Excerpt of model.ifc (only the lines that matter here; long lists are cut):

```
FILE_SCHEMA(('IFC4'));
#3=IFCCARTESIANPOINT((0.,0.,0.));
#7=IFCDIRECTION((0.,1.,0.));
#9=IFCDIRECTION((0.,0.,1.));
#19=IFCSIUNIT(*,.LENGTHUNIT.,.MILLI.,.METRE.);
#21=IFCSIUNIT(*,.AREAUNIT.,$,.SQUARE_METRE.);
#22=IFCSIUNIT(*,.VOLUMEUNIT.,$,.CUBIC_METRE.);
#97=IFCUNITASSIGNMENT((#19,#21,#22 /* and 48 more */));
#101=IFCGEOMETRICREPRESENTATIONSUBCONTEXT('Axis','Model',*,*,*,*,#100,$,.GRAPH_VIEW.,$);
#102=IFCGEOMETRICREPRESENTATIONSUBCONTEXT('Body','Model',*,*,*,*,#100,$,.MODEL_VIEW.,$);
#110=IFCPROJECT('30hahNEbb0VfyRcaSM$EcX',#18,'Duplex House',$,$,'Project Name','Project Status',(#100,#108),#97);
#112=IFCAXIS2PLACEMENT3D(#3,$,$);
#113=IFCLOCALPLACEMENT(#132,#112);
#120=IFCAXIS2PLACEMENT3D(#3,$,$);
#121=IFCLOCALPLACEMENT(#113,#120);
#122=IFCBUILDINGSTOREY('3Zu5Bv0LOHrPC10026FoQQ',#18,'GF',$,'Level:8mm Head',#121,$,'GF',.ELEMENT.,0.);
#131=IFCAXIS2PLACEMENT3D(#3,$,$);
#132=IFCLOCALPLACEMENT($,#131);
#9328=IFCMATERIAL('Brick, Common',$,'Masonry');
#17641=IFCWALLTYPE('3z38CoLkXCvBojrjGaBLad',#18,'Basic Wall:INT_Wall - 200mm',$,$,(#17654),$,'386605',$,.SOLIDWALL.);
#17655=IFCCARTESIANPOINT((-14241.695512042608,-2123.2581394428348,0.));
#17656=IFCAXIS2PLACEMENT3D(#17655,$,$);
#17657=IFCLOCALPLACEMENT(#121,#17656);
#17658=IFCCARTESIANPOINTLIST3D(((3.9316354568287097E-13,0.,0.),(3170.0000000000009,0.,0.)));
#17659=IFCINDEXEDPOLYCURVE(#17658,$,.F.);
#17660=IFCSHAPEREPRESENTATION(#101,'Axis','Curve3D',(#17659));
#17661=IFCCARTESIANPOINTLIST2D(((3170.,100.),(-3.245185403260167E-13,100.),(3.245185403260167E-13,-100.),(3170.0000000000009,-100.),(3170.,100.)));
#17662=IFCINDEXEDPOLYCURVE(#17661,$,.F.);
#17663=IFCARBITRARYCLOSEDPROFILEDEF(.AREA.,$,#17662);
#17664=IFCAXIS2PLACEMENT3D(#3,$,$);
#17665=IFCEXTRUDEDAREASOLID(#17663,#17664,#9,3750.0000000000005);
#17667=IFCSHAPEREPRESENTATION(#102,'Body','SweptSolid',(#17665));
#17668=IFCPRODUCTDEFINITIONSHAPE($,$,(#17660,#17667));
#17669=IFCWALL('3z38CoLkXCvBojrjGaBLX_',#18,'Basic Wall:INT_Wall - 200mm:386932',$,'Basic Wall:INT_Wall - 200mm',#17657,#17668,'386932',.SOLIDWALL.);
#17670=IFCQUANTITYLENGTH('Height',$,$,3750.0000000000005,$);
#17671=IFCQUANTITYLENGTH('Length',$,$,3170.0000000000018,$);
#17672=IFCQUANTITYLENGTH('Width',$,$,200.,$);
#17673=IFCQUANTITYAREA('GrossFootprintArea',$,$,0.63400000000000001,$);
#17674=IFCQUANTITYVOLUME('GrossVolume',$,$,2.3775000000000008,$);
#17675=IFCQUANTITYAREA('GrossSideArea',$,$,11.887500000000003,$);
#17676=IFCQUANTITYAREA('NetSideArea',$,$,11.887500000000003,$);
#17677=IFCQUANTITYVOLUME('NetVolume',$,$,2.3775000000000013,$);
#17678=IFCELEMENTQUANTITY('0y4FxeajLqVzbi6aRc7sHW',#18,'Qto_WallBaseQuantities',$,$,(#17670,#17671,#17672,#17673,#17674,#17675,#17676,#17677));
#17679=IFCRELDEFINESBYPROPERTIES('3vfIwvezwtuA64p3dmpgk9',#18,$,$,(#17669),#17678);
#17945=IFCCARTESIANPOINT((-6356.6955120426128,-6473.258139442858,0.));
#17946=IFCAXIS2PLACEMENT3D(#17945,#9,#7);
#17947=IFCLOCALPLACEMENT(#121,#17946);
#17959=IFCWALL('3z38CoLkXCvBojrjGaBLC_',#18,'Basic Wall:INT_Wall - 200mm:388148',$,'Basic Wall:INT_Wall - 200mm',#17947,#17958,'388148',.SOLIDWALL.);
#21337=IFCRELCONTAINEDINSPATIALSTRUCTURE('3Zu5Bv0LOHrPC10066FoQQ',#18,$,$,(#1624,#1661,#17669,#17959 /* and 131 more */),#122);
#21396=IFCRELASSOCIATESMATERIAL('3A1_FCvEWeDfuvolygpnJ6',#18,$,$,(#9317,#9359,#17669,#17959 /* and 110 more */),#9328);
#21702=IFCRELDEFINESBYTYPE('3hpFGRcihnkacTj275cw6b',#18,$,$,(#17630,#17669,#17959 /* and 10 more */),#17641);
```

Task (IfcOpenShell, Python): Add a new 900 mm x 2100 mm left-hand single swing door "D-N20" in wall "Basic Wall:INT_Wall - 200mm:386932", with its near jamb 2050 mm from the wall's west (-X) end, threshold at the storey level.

```python
import numpy as np
import ifcopenshell
import ifcopenshell.api.feature
import ifcopenshell.api.geometry
import ifcopenshell.api.pset
import ifcopenshell.api.root
import ifcopenshell.api.spatial
import ifcopenshell.geom
import ifcopenshell.util.element
import ifcopenshell.util.placement
import ifcopenshell.util.representation
import ifcopenshell.util.shape
import ifcopenshell.util.unit

model = ifcopenshell.open("model.ifc")
unit_scale = ifcopenshell.util.unit.calculate_unit_scale(model)
area_scale = ifcopenshell.util.unit.calculate_unit_scale(model, "AREAUNIT")
volume_scale = ifcopenshell.util.unit.calculate_unit_scale(model, "VOLUMEUNIT")
settings = ifcopenshell.geom.settings()


def volume(element):
    """Net volume in cubic metres, openings subtracted."""
    shape = ifcopenshell.geom.create_shape(settings, element)
    return ifcopenshell.util.shape.get_volume(shape.geometry)


wall = model.by_guid("3z38CoLkXCvBojrjGaBLX_")
storey = ifcopenshell.util.element.get_container(wall, ifc_class="IfcBuildingStorey")
context = ifcopenshell.util.representation.get_context(model, "Model", "Body", "MODEL_VIEW")
before = volume(wall)

width, height, from_end, sill = 0.9, 2.1, 2.05, 0.0  # metres

# The wall runs along its own X axis, and the end named is its -X end.
wall_shape = ifcopenshell.geom.create_shape(settings, wall)
x, y, z = ifcopenshell.util.shape.get_vertices(wall_shape.geometry).T
start = x.min() + from_end
face, thickness = float(y.min()), float(y.max() - y.min())
wall_matrix = ifcopenshell.util.placement.get_local_placement(wall.ObjectPlacement)
level = ifcopenshell.util.placement.get_local_placement(storey.ObjectPlacement)[2, 3]


def in_wall(x, y):
    """Placement at x, y metres in the wall's axes, at sill height."""
    matrix = wall_matrix.copy()
    matrix[:, 3] = wall_matrix @ np.array([x / unit_scale, y / unit_scale, 0.0, 1.0])
    matrix[2, 3] = level + sill / unit_scale
    return matrix


# Opening: a box that overshoots both wall faces by 50 mm.
opening = ifcopenshell.api.root.create_entity(model, ifc_class="IfcOpeningElement", predefined_type="OPENING")
box = ifcopenshell.api.geometry.add_wall_representation(
    model, context=context, length=width, height=height, thickness=thickness + 0.1
)
ifcopenshell.api.geometry.assign_representation(model, product=opening, representation=box)
ifcopenshell.api.geometry.edit_object_placement(model, product=opening, matrix=in_wall(start, face - 0.05), is_si=False)
ifcopenshell.api.feature.add_feature(model, feature=opening, element=wall)

door = ifcopenshell.api.root.create_entity(model, ifc_class="IfcDoor", name="D-N20", predefined_type="DOOR")
door.OverallWidth, door.OverallHeight = width / unit_scale, height / unit_scale
door.OperationType = "SINGLE_SWING_LEFT"
body = ifcopenshell.api.geometry.add_door_representation(
    model,
    context=context,
    overall_width=door.OverallWidth,
    overall_height=door.OverallHeight,
    operation_type="SINGLE_SWING_LEFT",
    lining_properties={"LiningDepth": thickness / unit_scale, "ThresholdDepth": thickness / unit_scale},
)
ifcopenshell.api.geometry.assign_representation(model, product=door, representation=body)
ifcopenshell.api.spatial.assign_container(model, products=[door], relating_structure=storey)
ifcopenshell.api.feature.add_filling(model, opening=opening, element=door)

# The lining spans the wall, so the door starts at the wall face.
ifcopenshell.api.geometry.edit_object_placement(model, product=door, matrix=in_wall(start, face), is_si=False)

after = volume(wall)

# Update the wall's stored quantities.
qto = model.by_id(ifcopenshell.util.element.get_pset(wall, "Qto_WallBaseQuantities", should_inherit=False)["id"])
ifcopenshell.api.pset.edit_qto(model, qto=qto, properties={
    "NetSideArea": after / thickness / area_scale,
    "NetVolume": after / volume_scale,
})

print(f"wall volume {before:.3f} -> {after:.3f} m3")

model.write("model_v2.ifc")
```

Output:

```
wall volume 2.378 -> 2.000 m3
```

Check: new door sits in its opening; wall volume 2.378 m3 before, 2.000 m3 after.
